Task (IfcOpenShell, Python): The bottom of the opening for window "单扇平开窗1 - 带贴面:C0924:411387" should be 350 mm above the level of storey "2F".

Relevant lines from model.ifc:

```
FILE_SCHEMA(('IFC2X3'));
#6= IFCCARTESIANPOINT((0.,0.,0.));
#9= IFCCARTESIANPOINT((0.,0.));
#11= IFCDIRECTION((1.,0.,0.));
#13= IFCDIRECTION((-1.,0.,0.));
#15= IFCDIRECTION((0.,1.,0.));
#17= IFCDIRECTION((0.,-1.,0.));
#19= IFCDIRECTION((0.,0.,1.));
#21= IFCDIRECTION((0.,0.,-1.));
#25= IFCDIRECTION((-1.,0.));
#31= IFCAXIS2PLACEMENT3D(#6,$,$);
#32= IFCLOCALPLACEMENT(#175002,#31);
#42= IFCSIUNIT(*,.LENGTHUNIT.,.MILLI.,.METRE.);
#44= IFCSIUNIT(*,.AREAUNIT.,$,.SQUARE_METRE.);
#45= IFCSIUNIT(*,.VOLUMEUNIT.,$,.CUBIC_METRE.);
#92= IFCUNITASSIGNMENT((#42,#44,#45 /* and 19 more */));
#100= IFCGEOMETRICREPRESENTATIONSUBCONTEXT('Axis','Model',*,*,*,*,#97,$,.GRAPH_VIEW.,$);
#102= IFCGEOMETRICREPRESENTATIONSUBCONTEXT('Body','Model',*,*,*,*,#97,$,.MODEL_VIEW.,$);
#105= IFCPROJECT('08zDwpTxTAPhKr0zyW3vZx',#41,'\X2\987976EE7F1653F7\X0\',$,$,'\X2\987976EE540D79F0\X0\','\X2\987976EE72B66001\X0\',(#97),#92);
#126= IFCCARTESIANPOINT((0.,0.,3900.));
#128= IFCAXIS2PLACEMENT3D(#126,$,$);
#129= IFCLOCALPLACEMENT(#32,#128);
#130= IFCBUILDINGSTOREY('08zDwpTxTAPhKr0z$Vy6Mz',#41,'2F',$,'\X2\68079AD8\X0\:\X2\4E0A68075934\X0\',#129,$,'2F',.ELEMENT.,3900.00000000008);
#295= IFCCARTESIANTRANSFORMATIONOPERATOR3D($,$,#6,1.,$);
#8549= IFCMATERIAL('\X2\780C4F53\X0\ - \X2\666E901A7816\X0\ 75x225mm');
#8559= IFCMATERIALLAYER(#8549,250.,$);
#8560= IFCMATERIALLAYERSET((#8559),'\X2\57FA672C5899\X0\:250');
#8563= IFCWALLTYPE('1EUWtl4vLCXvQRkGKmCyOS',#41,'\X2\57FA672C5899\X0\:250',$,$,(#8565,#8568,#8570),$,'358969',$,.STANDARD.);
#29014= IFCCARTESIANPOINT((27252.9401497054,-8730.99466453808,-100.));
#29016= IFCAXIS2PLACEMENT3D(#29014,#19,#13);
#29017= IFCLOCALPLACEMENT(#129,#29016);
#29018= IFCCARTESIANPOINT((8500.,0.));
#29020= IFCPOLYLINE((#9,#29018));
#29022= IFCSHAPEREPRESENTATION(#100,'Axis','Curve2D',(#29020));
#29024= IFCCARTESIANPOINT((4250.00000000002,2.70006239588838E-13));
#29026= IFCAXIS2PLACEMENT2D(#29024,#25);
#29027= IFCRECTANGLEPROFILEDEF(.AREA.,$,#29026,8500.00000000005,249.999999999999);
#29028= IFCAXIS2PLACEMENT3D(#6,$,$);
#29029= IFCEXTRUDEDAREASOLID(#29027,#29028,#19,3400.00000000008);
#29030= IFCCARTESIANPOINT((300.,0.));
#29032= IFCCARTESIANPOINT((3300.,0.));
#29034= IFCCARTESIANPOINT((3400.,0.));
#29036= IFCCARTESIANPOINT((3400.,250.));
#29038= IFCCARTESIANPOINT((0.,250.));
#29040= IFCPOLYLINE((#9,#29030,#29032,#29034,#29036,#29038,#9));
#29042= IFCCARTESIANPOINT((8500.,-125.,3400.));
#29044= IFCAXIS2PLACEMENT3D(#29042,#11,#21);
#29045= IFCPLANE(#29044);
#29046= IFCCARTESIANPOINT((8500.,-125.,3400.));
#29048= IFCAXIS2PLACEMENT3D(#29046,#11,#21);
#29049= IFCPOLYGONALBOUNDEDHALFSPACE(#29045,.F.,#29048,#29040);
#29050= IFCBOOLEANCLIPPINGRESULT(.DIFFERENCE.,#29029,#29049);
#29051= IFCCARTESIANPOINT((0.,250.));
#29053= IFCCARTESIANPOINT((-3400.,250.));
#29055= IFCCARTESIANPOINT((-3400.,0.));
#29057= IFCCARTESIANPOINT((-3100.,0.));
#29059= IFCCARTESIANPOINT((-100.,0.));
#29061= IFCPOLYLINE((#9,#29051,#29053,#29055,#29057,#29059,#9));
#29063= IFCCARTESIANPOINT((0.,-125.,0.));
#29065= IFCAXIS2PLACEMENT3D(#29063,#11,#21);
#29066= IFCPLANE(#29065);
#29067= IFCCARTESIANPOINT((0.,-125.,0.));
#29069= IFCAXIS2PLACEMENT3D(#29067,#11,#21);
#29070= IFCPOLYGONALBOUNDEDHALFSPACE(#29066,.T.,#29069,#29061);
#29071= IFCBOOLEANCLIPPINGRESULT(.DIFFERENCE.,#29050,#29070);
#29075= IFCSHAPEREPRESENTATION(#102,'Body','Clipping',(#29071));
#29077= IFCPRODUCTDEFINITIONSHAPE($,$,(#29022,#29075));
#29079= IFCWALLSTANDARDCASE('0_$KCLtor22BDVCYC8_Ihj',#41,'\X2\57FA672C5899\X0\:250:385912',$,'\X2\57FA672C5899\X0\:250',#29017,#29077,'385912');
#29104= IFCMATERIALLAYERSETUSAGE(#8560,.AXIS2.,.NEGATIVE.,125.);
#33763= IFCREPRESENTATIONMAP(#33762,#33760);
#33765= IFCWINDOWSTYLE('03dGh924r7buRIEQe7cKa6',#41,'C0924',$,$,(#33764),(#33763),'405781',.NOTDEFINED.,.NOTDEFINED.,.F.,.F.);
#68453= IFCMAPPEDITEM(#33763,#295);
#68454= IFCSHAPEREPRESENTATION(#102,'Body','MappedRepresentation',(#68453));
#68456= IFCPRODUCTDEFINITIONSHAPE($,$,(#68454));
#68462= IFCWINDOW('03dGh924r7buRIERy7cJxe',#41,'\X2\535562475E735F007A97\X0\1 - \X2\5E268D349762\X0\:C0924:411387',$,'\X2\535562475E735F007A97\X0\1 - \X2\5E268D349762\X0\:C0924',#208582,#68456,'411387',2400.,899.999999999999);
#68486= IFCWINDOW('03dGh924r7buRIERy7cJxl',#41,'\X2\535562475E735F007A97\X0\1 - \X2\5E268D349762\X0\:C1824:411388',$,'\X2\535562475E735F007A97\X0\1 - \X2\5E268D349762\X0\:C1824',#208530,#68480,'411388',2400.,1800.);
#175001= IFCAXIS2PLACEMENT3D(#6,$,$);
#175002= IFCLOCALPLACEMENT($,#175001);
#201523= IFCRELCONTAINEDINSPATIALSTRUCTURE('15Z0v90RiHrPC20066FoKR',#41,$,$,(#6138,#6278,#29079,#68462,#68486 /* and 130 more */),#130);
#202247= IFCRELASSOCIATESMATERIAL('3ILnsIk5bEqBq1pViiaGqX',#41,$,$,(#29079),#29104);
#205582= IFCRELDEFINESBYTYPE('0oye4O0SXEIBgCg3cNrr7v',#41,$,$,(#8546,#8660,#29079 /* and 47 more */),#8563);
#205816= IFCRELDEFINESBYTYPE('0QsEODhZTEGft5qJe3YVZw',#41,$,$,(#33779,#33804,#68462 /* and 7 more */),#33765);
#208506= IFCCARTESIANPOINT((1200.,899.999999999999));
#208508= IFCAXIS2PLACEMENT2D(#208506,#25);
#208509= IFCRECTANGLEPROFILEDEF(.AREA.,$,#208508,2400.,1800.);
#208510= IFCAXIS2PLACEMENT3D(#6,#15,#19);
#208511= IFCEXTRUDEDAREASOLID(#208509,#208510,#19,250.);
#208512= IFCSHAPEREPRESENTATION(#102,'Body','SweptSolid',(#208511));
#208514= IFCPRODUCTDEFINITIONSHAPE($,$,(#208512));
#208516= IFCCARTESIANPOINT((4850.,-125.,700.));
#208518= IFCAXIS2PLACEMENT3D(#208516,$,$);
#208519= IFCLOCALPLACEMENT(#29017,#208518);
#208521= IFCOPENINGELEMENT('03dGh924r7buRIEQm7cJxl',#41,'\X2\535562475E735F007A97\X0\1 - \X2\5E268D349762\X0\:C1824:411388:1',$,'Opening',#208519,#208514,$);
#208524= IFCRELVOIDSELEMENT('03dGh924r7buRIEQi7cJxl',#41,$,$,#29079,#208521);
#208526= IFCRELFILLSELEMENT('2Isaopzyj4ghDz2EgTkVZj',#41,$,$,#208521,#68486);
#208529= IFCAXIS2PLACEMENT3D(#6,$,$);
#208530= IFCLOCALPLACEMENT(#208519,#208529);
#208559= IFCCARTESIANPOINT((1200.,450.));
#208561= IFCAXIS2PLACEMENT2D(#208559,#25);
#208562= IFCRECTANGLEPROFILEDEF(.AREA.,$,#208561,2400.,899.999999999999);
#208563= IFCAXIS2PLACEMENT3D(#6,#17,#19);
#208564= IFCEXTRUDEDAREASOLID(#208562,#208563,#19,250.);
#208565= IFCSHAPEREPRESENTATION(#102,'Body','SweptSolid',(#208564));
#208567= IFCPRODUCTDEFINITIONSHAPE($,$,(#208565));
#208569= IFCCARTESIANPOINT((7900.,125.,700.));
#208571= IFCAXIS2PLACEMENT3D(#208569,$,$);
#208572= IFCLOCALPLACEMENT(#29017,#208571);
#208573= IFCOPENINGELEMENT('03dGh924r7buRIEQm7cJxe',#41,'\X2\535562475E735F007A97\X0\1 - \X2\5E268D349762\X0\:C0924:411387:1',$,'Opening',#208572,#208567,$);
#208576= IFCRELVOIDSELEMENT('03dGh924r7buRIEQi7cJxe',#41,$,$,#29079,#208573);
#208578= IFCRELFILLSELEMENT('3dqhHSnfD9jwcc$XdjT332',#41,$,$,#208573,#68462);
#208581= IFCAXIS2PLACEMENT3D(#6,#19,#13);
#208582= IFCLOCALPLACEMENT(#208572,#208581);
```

```python
import numpy as np
import ifcopenshell
import ifcopenshell.api.geometry
import ifcopenshell.geom
import ifcopenshell.util.element
import ifcopenshell.util.placement
import ifcopenshell.util.shape
import ifcopenshell.util.unit

model = ifcopenshell.open("model.ifc")
unit_scale = ifcopenshell.util.unit.calculate_unit_scale(model)

window = model.by_guid("03dGh924r7buRIERy7cJxe")
opening = window.FillsVoids[0].RelatingOpeningElement
storey = ifcopenshell.util.element.get_container(window, ifc_class="IfcBuildingStorey")
level = ifcopenshell.util.placement.get_local_placement(storey.ObjectPlacement)[2, 3]

# The opening's origin need not be at the sill, so measure its lowest point.
shape = ifcopenshell.geom.create_shape(ifcopenshell.geom.settings(), opening)
bottom = ifcopenshell.util.shape.get_shape_bottom_elevation(shape, shape.geometry) / unit_scale
dz = level + 0.35 / unit_scale - bottom

shift = np.array([0.0, 0.0, dz])
# The window is placed relative to its opening, so it follows when the opening moves.
matrix = ifcopenshell.util.placement.get_local_placement(opening.ObjectPlacement)
matrix[:3, 3] += shift
ifcopenshell.api.geometry.edit_object_placement(
    model, product=opening, matrix=matrix, is_si=False, should_transform_children=True
)

print(f"moved by {dz * unit_scale:+.3f} m")

model.write("model_updated.ifc")
```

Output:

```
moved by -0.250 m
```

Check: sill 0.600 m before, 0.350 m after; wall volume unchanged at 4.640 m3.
